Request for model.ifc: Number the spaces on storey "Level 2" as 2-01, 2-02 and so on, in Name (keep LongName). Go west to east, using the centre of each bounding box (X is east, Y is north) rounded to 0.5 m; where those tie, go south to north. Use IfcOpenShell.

First a look at what the model holds.

```python
import ifcopenshell
import ifcopenshell.util.element
import ifcopenshell.util.placement

model = ifcopenshell.open("model.ifc")
print(model.schema)
storey = next(s for s in model.by_type("IfcBuildingStorey") if s.Name == "Level 2")
spaces = [e for e in ifcopenshell.util.element.get_decomposition(storey) if e.is_a("IfcSpace")]
for e in sorted(spaces, key=lambda e: e.id()):
    origin = ifcopenshell.util.placement.get_local_placement(e.ObjectPlacement)[:3, 3]
    print(e.id(), e.Name, e.LongName, origin.round(2) + 0.0, sep=" | ")
```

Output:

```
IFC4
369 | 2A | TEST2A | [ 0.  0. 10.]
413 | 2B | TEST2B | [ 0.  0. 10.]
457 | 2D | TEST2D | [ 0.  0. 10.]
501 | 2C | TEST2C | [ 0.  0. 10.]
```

```python
import ifcopenshell
import ifcopenshell.geom
import ifcopenshell.util.element
import ifcopenshell.util.shape

model = ifcopenshell.open("model.ifc")
settings = ifcopenshell.geom.settings()
settings.set("use-world-coords", True)


def centre(element):
    shape = ifcopenshell.geom.create_shape(settings, element)
    return ifcopenshell.util.shape.get_bbox_centroid(shape.geometry)


storey = next(s for s in model.by_type("IfcBuildingStorey") if s.Name == "Level 2")
spaces = [e for e in ifcopenshell.util.element.get_decomposition(storey) if e.is_a("IfcSpace")]

# Insertion points can sit at a corner or the storey origin, so sort by the geometry (in metres).
centres = {e: centre(e) for e in spaces}
spaces.sort(key=lambda e: (round(centres[e][0] / 0.5), centres[e][1]))

for i, e in enumerate(spaces, start=1):
    number = f"2-{i:02d}"
    e.Name = number
    print(e.id(), number)

model.write("model-out.ifc")
```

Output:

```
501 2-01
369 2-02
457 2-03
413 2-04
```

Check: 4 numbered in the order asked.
